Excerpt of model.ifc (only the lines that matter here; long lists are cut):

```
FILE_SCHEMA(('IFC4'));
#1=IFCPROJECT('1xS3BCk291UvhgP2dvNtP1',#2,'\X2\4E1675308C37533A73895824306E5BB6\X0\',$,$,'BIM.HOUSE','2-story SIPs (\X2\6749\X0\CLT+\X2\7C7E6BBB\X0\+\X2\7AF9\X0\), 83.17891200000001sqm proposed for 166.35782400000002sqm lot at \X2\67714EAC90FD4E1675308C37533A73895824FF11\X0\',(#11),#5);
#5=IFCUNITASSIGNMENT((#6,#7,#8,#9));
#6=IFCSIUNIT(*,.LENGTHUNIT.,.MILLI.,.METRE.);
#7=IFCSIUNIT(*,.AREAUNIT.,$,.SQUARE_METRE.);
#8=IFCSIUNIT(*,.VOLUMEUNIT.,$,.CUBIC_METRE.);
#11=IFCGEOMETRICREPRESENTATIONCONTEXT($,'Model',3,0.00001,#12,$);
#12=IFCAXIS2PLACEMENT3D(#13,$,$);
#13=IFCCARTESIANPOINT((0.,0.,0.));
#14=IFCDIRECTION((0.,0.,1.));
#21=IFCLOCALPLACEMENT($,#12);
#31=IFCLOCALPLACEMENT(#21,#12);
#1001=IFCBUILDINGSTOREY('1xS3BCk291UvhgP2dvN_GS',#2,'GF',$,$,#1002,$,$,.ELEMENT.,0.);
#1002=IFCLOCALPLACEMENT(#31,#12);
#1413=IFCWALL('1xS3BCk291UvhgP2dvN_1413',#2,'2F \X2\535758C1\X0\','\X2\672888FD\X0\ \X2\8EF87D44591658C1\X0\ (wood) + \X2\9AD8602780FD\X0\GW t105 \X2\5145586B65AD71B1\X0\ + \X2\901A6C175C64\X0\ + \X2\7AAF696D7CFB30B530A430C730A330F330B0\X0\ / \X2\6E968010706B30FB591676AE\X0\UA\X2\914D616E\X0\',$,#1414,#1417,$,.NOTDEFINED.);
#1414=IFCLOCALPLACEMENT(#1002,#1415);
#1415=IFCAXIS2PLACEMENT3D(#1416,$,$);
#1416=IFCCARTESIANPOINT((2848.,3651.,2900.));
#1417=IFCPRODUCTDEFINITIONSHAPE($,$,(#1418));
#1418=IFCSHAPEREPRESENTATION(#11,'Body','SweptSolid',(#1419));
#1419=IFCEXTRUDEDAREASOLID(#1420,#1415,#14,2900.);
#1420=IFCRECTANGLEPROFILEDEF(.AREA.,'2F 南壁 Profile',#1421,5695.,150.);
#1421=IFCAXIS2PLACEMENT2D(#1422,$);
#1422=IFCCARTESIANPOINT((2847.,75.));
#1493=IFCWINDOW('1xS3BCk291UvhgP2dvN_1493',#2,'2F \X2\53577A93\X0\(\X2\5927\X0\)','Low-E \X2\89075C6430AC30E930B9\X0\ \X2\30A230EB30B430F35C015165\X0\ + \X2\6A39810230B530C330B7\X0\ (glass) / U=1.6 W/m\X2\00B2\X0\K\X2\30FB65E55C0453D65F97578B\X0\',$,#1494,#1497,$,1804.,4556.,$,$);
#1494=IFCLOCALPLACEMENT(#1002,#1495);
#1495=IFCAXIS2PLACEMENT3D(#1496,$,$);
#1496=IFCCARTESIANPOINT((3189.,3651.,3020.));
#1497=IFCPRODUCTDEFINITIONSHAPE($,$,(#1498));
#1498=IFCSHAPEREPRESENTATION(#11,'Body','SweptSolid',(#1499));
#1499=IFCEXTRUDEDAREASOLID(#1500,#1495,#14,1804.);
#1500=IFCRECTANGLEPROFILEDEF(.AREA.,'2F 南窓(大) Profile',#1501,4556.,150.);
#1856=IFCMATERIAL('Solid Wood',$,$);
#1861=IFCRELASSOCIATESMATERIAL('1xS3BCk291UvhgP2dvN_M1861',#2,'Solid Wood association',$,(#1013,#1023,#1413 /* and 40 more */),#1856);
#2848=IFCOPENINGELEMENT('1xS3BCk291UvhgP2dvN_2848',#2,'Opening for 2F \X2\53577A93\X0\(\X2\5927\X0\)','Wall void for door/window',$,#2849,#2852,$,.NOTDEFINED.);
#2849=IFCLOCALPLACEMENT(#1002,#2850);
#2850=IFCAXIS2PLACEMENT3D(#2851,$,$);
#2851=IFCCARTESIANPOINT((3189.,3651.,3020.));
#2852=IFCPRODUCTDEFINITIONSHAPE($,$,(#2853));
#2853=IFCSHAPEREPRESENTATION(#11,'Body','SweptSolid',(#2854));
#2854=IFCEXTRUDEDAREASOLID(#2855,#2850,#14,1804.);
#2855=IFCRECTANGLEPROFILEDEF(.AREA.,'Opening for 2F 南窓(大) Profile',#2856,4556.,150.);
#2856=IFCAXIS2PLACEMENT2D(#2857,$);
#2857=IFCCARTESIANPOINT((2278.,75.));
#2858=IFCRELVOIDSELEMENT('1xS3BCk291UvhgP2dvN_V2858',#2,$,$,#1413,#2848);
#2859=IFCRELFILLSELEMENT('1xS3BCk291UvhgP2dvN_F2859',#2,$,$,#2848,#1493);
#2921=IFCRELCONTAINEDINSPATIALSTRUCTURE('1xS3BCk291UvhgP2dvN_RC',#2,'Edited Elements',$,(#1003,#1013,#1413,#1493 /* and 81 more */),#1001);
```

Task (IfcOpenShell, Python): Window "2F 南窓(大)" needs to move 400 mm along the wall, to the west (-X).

```python
import ifcopenshell
import ifcopenshell.api.geometry
import ifcopenshell.util.placement

model = ifcopenshell.open("model.ifc")

window = model.by_guid("1xS3BCk291UvhgP2dvN_1493")
opening = window.FillsVoids[0].RelatingOpeningElement
wall = opening.VoidsElements[0].RelatingBuildingElement

wall_matrix = ifcopenshell.util.placement.get_local_placement(wall.ObjectPlacement)
shift = wall_matrix[:3, 0] * -400.0
before = ifcopenshell.util.placement.get_local_placement(window.ObjectPlacement)[:3, 3].copy()

# The window is not placed relative to its opening, so move both.
for product in (opening, window):
    matrix = ifcopenshell.util.placement.get_local_placement(product.ObjectPlacement)
    matrix[:3, 3] += shift
    ifcopenshell.api.geometry.edit_object_placement(model, product=product, matrix=matrix, is_si=False)

after = ifcopenshell.util.placement.get_local_placement(window.ObjectPlacement)[:3, 3]
print("window moved by", (after - before).round(3) + 0.0)

model.write("model-out.ifc")
```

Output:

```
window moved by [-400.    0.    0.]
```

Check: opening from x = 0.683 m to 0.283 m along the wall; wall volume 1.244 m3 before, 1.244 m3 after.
